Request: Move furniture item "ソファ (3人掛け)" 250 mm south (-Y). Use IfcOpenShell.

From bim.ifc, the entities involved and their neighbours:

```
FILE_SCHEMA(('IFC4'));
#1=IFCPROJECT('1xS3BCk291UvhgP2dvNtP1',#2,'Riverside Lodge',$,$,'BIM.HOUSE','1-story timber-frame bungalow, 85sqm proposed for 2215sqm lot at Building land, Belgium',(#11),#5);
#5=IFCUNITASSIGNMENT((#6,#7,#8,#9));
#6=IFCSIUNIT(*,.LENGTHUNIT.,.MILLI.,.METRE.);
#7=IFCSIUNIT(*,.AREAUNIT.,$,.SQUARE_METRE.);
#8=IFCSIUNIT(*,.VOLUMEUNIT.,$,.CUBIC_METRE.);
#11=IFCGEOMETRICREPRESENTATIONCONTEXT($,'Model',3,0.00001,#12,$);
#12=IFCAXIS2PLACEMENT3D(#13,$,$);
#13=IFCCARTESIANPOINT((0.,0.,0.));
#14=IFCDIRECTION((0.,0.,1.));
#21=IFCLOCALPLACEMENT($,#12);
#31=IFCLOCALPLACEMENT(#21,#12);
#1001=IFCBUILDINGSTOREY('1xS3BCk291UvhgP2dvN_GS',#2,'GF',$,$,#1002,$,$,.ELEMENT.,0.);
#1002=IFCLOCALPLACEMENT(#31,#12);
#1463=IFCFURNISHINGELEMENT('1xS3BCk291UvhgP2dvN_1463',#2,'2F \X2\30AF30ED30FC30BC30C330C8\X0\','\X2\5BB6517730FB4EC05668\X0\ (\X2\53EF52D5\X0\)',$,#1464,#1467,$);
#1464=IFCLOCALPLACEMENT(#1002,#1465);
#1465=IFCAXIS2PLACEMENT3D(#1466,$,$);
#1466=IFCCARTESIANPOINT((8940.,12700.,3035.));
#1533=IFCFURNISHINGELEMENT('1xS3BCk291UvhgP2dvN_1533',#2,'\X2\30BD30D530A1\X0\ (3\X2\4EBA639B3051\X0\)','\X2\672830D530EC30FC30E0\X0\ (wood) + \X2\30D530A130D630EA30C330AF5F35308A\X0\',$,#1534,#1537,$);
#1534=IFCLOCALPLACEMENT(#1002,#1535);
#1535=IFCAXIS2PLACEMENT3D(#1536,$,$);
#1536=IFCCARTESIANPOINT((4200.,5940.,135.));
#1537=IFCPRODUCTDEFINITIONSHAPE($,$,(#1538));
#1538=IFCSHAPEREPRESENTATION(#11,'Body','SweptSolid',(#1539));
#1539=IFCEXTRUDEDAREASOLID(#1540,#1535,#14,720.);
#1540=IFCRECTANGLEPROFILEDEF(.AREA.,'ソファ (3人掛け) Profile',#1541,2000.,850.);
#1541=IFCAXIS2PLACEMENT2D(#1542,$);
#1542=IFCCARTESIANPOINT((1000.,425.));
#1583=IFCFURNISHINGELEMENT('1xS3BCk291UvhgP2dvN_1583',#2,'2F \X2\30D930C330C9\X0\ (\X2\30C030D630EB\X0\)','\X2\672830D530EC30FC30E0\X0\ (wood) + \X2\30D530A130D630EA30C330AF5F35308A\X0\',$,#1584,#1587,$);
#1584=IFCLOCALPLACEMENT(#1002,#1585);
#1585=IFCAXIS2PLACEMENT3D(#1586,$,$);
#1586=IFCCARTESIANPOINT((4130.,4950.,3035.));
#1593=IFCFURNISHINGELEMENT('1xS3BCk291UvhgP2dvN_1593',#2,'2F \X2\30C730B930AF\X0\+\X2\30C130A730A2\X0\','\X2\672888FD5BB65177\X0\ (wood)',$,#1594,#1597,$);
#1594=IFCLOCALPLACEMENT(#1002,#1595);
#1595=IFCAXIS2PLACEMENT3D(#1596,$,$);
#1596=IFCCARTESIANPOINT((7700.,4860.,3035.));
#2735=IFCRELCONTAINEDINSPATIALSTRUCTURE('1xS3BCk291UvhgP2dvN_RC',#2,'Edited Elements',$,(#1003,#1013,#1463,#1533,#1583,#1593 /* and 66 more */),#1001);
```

```python
import ifcopenshell
import ifcopenshell.api.geometry
import ifcopenshell.util.placement
import ifcopenshell.util.unit

model = ifcopenshell.open("bim.ifc")
unit_scale = ifcopenshell.util.unit.calculate_unit_scale(model)

item = model.by_guid("1xS3BCk291UvhgP2dvN_1533")
matrix = ifcopenshell.util.placement.get_local_placement(item.ObjectPlacement)
matrix[1, 3] -= 0.25 / unit_scale
ifcopenshell.api.geometry.edit_object_placement(model, product=item, matrix=matrix, is_si=False)

print(ifcopenshell.util.placement.get_local_placement(item.ObjectPlacement).round(3) + 0.0)

model.write("bim_rev.ifc")
```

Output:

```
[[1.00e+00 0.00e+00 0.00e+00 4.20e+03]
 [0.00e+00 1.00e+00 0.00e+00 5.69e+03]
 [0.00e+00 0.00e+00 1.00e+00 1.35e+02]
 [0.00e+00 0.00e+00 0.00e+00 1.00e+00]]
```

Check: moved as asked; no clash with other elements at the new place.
